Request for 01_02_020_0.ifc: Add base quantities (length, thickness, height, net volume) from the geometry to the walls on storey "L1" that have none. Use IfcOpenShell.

First a look at what the model holds.

```python
import ifcopenshell
import ifcopenshell.util.element
import ifcopenshell.util.unit

model = ifcopenshell.open("01_02_020_0.ifc")
print(model.schema)
for unit_type in ("LENGTHUNIT", "AREAUNIT", "VOLUMEUNIT"):
    print(unit_type, ifcopenshell.util.unit.calculate_unit_scale(model, unit_type))
storey = next(s for s in model.by_type("IfcBuildingStorey") if s.Name == "L1")
walls = [e for e in ifcopenshell.util.element.get_decomposition(storey) if e.is_a("IfcWall")]
for e in sorted(walls, key=lambda e: e.id()):
    print(e.id(), e.is_a(), e.Name, list(ifcopenshell.util.element.get_psets(e, qtos_only=True)), sep=" | ")
```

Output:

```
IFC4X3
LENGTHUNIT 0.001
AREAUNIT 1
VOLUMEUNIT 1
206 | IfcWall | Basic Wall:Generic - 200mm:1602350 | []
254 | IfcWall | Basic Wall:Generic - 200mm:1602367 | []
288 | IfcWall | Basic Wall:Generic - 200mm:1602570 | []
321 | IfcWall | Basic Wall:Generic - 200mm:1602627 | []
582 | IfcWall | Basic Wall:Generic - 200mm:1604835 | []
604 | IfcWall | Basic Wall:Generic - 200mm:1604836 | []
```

```python
import ifcopenshell
import ifcopenshell.api.pset
import ifcopenshell.geom
import ifcopenshell.util.element
import ifcopenshell.util.shape
import ifcopenshell.util.unit

model = ifcopenshell.open("01_02_020_0.ifc")
unit_scale = ifcopenshell.util.unit.calculate_unit_scale(model)
volume_scale = ifcopenshell.util.unit.calculate_unit_scale(model, "VOLUMEUNIT")
settings = ifcopenshell.geom.settings()

storey = next(s for s in model.by_type("IfcBuildingStorey") if s.Name == "L1")
walls = [e for e in ifcopenshell.util.element.get_decomposition(storey) if e.is_a("IfcWall")]

for e in sorted(walls, key=lambda e: e.id()):
    if ifcopenshell.util.element.get_psets(e, qtos_only=True, should_inherit=False):
        continue
    # Geometry comes back in metres, in the element's own axes.
    shape = ifcopenshell.geom.create_shape(settings, e)
    values = {
        "Length": ifcopenshell.util.shape.get_x(shape.geometry) / unit_scale,
        "Width": ifcopenshell.util.shape.get_y(shape.geometry) / unit_scale,
        "Height": ifcopenshell.util.shape.get_z(shape.geometry) / unit_scale,
        "NetVolume": ifcopenshell.util.shape.get_volume(shape.geometry) / volume_scale,
    }
    qto = ifcopenshell.api.pset.add_qto(model, product=e, name="Qto_WallBaseQuantities")
    ifcopenshell.api.pset.edit_qto(model, qto=qto, properties=values)
    print(e.id(), {k: round(v, 3) for k, v in values.items()})

model.write("01_02_020_0_edited.ifc")
```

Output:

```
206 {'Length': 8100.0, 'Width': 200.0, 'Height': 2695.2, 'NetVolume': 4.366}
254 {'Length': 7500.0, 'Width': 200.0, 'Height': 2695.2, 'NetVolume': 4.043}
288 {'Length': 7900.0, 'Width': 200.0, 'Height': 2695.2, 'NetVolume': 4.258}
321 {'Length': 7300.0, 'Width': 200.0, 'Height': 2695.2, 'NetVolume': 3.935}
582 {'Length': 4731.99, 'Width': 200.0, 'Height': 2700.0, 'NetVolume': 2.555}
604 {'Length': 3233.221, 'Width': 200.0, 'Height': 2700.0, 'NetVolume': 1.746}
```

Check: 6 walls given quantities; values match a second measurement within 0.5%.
